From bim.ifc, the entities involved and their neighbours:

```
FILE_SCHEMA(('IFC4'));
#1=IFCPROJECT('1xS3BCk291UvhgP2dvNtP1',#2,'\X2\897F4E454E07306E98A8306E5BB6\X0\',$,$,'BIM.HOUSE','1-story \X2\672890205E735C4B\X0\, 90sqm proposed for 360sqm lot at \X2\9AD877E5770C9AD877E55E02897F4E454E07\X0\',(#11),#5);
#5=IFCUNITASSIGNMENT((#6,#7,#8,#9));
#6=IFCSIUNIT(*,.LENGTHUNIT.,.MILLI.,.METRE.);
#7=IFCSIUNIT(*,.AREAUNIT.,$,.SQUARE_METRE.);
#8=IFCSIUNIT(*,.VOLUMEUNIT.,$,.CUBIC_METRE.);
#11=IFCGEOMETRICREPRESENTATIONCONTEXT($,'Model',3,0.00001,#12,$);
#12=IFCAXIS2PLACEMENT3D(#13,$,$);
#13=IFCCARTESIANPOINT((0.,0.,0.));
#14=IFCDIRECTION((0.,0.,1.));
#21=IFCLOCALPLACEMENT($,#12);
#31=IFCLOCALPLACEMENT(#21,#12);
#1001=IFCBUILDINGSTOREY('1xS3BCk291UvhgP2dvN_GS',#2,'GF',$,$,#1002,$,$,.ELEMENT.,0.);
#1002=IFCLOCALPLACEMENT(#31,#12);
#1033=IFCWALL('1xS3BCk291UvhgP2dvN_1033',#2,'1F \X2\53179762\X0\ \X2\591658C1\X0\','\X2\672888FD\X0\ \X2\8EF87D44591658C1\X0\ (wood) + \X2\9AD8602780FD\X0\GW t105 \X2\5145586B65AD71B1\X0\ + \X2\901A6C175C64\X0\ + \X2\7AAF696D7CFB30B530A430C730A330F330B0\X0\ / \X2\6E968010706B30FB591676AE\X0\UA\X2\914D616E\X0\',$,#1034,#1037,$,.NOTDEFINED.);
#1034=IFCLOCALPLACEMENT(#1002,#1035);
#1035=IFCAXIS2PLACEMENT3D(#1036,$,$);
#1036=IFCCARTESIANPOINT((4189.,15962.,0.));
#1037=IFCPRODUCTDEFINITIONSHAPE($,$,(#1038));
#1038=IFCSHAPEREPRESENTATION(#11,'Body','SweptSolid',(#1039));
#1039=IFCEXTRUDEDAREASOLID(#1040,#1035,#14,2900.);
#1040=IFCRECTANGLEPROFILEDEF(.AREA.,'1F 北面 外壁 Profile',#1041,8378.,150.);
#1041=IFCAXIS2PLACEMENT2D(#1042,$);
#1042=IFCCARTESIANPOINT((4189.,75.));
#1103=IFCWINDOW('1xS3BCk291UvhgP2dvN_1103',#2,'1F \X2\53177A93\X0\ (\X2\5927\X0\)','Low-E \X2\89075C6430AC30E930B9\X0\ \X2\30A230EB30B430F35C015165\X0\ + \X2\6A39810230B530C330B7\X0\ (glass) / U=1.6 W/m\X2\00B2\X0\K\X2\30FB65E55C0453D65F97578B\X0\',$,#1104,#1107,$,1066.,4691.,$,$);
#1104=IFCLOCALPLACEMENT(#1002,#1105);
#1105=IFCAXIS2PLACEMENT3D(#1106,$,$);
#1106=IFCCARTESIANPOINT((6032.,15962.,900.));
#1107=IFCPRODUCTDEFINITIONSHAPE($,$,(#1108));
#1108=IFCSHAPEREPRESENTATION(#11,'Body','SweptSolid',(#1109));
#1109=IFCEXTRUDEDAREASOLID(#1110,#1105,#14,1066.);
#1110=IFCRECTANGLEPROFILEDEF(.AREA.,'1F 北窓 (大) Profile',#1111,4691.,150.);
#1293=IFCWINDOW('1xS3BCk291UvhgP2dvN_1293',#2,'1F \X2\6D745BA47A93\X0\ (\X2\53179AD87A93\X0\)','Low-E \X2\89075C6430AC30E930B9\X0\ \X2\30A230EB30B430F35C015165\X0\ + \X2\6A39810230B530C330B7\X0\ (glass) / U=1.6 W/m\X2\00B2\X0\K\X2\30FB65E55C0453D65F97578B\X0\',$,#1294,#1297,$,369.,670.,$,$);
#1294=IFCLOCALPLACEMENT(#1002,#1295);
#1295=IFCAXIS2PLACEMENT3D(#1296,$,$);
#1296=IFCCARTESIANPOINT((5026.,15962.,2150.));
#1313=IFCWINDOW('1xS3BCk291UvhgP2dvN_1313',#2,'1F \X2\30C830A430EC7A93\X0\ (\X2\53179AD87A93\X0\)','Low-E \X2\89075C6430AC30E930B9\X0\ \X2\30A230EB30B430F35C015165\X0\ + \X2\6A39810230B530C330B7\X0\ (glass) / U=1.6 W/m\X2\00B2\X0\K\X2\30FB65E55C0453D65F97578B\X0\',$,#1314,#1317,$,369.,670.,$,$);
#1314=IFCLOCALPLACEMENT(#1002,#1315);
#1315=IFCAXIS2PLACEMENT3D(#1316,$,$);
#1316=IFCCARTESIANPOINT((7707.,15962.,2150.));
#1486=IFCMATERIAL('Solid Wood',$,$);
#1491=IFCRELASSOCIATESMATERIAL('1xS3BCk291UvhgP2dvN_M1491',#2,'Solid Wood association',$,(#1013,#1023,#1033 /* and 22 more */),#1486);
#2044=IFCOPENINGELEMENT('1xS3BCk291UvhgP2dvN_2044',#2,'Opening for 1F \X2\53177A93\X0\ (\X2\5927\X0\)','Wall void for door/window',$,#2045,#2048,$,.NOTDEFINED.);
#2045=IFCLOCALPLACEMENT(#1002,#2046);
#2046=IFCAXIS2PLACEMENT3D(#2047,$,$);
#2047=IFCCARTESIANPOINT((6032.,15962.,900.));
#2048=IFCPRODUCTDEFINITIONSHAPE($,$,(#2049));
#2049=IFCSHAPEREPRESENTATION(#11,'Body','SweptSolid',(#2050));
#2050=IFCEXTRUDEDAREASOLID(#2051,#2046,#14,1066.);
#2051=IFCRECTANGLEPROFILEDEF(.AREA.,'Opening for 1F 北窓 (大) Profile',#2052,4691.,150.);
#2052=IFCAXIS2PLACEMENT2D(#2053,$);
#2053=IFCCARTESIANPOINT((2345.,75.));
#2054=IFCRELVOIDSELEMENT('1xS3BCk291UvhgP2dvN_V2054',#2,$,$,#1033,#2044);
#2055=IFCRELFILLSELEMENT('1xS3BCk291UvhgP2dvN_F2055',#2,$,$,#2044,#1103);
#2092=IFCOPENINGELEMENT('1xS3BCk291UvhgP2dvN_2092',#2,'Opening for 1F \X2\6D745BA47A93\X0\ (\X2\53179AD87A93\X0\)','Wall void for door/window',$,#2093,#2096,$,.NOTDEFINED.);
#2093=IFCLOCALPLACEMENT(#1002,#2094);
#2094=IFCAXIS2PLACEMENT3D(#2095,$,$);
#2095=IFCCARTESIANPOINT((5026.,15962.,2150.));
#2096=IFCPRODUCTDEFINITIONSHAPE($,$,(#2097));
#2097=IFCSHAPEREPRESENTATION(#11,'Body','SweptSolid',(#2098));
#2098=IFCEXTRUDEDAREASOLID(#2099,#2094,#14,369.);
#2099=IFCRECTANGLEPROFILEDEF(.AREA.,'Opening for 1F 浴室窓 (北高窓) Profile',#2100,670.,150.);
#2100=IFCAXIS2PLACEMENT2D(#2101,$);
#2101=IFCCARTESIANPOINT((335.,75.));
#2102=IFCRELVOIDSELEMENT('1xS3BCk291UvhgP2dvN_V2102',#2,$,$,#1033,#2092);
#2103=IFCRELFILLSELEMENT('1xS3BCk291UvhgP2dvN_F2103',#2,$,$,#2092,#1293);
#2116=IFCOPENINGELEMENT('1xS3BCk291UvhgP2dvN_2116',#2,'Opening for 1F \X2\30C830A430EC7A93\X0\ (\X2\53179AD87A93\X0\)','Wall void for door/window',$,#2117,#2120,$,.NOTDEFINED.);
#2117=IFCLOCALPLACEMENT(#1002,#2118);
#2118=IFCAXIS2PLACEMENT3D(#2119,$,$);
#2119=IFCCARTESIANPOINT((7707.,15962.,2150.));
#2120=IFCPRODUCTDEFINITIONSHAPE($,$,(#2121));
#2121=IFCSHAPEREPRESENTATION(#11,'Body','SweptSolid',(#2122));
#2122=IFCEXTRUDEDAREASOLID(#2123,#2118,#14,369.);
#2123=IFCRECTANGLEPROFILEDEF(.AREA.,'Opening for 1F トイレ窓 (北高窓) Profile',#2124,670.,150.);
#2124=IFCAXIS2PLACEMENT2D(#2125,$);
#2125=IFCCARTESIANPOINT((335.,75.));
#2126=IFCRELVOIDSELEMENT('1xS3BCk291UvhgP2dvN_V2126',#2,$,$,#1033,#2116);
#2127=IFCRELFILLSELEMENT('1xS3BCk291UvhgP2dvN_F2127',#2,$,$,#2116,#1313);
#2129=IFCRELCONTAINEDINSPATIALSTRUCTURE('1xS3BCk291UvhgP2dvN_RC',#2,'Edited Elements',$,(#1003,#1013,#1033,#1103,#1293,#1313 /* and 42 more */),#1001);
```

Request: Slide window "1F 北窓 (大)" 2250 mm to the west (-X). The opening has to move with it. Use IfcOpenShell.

```python
import ifcopenshell
import ifcopenshell.api.geometry
import ifcopenshell.util.placement
import ifcopenshell.util.unit

model = ifcopenshell.open("bim.ifc")
unit_scale = ifcopenshell.util.unit.calculate_unit_scale(model)

window = model.by_guid("1xS3BCk291UvhgP2dvN_1103")
opening = window.FillsVoids[0].RelatingOpeningElement
wall = opening.VoidsElements[0].RelatingBuildingElement

wall_matrix = ifcopenshell.util.placement.get_local_placement(wall.ObjectPlacement)
shift = wall_matrix[:3, 0] * -2.25 / unit_scale
before = ifcopenshell.util.placement.get_local_placement(window.ObjectPlacement)[:3, 3].copy()

# The window is not placed relative to its opening, so move both.
for product in (opening, window):
    matrix = ifcopenshell.util.placement.get_local_placement(product.ObjectPlacement)
    matrix[:3, 3] += shift
    ifcopenshell.api.geometry.edit_object_placement(model, product=product, matrix=matrix, is_si=False)

after = ifcopenshell.util.placement.get_local_placement(window.ObjectPlacement)[:3, 3]
print("window moved by", (after - before).round(3) + 0.0)

model.write("bim_edited.ifc")
```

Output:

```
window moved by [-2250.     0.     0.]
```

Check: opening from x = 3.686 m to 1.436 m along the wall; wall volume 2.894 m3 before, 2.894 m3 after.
